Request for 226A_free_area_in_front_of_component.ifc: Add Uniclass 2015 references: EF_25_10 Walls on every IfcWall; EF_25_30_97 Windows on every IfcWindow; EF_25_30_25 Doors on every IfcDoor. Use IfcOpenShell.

First a look at what the model holds.

```python
import ifcopenshell

model = ifcopenshell.open("226A_free_area_in_front_of_component.ifc")
print(model.schema)
print("classifications:", [c.Name for c in model.by_type("IfcClassification")])
for ifc_class in ("IfcDoor", "IfcRoof", "IfcStair", "IfcWall", "IfcWindow"):
    print(ifc_class, len(model.by_type(ifc_class)))
```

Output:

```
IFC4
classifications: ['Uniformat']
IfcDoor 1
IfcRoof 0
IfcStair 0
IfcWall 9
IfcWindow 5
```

```python
import ifcopenshell
import ifcopenshell.api.classification

model = ifcopenshell.open("226A_free_area_in_front_of_component.ifc")

system = ifcopenshell.api.classification.add_classification(model, classification="Uniclass 2015")

codes = {
    "IfcWall": ("EF_25_10", "Walls"),
    "IfcWindow": ("EF_25_30_97", "Windows"),
    "IfcDoor": ("EF_25_30_25", "Doors"),
}
for ifc_class, (code, name) in codes.items():
    products = model.by_type(ifc_class)
    ifcopenshell.api.classification.add_reference(
        model, products=products, classification=system, identification=code, name=name
    )
    print(code, len(products))

model.write("226A_free_area_in_front_of_component_v2.ifc")
```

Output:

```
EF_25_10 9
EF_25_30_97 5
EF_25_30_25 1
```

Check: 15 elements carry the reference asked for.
